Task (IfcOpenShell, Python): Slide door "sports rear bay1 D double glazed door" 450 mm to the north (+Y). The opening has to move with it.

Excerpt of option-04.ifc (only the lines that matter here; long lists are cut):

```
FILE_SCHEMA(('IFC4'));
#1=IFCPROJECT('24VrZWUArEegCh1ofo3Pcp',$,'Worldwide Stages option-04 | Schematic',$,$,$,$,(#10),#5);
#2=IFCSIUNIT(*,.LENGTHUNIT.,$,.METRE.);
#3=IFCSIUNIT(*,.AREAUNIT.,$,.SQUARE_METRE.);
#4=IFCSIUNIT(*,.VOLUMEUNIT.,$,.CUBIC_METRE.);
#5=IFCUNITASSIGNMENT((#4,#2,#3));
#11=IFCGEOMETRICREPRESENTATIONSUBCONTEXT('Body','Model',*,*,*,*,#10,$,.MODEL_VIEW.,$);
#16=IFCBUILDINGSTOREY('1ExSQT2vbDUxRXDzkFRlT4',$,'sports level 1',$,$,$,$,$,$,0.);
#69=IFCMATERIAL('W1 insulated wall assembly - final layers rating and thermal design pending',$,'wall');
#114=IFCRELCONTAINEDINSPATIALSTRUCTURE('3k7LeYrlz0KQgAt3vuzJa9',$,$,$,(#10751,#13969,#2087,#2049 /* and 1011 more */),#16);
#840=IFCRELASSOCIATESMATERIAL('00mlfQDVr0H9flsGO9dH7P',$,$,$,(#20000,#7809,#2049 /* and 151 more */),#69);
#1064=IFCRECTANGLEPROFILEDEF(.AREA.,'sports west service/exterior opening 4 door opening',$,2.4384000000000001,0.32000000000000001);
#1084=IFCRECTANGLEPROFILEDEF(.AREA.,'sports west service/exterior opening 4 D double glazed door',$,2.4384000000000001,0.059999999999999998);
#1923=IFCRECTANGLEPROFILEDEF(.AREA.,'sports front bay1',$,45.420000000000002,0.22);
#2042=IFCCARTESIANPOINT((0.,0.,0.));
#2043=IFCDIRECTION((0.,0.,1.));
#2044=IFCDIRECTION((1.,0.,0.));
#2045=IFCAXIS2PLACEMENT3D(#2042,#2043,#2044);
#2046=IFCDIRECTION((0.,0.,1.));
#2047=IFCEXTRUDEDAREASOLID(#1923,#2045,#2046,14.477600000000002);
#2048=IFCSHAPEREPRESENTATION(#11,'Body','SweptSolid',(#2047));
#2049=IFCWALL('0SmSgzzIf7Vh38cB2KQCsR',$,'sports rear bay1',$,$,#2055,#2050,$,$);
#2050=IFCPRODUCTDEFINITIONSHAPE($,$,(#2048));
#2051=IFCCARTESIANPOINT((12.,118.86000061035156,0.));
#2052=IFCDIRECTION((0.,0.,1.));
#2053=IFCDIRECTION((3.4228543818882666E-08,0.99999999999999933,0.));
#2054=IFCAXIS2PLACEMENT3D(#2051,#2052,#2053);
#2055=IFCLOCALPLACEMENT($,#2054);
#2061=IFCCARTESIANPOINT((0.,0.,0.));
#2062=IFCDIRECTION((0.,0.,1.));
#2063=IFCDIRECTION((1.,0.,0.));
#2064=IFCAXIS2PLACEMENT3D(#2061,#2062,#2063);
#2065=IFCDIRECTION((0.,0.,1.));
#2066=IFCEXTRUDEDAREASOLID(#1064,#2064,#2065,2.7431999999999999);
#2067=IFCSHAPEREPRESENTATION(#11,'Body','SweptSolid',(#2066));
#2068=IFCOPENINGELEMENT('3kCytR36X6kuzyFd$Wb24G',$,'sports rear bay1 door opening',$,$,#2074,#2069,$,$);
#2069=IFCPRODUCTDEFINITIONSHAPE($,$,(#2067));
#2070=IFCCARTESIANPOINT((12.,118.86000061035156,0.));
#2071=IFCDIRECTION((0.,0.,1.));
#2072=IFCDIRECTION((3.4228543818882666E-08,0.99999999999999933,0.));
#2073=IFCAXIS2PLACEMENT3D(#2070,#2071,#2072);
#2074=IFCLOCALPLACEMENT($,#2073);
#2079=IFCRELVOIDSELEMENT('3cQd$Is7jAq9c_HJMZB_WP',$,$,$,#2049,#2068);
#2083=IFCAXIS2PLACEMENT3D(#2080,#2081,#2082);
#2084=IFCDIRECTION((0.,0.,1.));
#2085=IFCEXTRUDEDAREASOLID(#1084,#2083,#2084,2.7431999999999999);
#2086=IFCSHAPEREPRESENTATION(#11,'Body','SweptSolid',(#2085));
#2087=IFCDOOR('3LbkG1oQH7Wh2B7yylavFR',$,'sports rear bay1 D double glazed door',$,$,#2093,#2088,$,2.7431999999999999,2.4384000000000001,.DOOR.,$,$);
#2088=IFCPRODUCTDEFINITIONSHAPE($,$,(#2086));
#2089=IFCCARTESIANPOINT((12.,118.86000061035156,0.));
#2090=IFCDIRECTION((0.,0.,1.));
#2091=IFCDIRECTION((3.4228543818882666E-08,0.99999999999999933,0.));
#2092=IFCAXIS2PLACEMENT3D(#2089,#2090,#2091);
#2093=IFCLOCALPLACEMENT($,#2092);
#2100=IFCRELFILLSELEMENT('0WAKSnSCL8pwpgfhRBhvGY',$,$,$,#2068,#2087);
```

```python
import ifcopenshell
import ifcopenshell.api.geometry
import ifcopenshell.util.placement
import ifcopenshell.util.unit

model = ifcopenshell.open("option-04.ifc")
unit_scale = ifcopenshell.util.unit.calculate_unit_scale(model)

door = model.by_guid("3LbkG1oQH7Wh2B7yylavFR")
opening = door.FillsVoids[0].RelatingOpeningElement
wall = opening.VoidsElements[0].RelatingBuildingElement

wall_matrix = ifcopenshell.util.placement.get_local_placement(wall.ObjectPlacement)
shift = wall_matrix[:3, 0] * 0.45 / unit_scale
before = ifcopenshell.util.placement.get_local_placement(door.ObjectPlacement)[:3, 3].copy()

# The door is not placed relative to its opening, so move both.
for product in (opening, door):
    matrix = ifcopenshell.util.placement.get_local_placement(product.ObjectPlacement)
    matrix[:3, 3] += shift
    ifcopenshell.api.geometry.edit_object_placement(model, product=product, matrix=matrix, is_si=False)

after = ifcopenshell.util.placement.get_local_placement(door.ObjectPlacement)[:3, 3]
print("door moved by", (after - before).round(3) + 0.0)

model.write("option-04_v2.ifc")
```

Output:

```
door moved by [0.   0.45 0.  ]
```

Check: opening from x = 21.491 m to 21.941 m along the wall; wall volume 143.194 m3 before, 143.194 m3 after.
